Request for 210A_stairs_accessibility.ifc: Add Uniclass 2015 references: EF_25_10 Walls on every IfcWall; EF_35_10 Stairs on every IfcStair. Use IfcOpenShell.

First a look at what the model holds.

```python
import ifcopenshell

model = ifcopenshell.open("210A_stairs_accessibility.ifc")
print(model.schema)
print("classifications:", [c.Name for c in model.by_type("IfcClassification")])
for ifc_class in ("IfcDoor", "IfcRoof", "IfcStair", "IfcWall", "IfcWindow"):
    print(ifc_class, len(model.by_type(ifc_class)))
```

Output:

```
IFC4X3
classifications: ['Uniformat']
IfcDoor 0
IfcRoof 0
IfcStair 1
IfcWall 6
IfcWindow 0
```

```python
import ifcopenshell
import ifcopenshell.api.classification

model = ifcopenshell.open("210A_stairs_accessibility.ifc")

system = ifcopenshell.api.classification.add_classification(model, classification="Uniclass 2015")

codes = {
    "IfcWall": ("EF_25_10", "Walls"),
    "IfcStair": ("EF_35_10", "Stairs"),
}
for ifc_class, (code, name) in codes.items():
    products = model.by_type(ifc_class)
    ifcopenshell.api.classification.add_reference(
        model, products=products, classification=system, identification=code, name=name
    )
    print(code, len(products))

model.write("210A_stairs_accessibility_v2.ifc")
```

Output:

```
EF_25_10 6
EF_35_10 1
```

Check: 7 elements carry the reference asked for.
